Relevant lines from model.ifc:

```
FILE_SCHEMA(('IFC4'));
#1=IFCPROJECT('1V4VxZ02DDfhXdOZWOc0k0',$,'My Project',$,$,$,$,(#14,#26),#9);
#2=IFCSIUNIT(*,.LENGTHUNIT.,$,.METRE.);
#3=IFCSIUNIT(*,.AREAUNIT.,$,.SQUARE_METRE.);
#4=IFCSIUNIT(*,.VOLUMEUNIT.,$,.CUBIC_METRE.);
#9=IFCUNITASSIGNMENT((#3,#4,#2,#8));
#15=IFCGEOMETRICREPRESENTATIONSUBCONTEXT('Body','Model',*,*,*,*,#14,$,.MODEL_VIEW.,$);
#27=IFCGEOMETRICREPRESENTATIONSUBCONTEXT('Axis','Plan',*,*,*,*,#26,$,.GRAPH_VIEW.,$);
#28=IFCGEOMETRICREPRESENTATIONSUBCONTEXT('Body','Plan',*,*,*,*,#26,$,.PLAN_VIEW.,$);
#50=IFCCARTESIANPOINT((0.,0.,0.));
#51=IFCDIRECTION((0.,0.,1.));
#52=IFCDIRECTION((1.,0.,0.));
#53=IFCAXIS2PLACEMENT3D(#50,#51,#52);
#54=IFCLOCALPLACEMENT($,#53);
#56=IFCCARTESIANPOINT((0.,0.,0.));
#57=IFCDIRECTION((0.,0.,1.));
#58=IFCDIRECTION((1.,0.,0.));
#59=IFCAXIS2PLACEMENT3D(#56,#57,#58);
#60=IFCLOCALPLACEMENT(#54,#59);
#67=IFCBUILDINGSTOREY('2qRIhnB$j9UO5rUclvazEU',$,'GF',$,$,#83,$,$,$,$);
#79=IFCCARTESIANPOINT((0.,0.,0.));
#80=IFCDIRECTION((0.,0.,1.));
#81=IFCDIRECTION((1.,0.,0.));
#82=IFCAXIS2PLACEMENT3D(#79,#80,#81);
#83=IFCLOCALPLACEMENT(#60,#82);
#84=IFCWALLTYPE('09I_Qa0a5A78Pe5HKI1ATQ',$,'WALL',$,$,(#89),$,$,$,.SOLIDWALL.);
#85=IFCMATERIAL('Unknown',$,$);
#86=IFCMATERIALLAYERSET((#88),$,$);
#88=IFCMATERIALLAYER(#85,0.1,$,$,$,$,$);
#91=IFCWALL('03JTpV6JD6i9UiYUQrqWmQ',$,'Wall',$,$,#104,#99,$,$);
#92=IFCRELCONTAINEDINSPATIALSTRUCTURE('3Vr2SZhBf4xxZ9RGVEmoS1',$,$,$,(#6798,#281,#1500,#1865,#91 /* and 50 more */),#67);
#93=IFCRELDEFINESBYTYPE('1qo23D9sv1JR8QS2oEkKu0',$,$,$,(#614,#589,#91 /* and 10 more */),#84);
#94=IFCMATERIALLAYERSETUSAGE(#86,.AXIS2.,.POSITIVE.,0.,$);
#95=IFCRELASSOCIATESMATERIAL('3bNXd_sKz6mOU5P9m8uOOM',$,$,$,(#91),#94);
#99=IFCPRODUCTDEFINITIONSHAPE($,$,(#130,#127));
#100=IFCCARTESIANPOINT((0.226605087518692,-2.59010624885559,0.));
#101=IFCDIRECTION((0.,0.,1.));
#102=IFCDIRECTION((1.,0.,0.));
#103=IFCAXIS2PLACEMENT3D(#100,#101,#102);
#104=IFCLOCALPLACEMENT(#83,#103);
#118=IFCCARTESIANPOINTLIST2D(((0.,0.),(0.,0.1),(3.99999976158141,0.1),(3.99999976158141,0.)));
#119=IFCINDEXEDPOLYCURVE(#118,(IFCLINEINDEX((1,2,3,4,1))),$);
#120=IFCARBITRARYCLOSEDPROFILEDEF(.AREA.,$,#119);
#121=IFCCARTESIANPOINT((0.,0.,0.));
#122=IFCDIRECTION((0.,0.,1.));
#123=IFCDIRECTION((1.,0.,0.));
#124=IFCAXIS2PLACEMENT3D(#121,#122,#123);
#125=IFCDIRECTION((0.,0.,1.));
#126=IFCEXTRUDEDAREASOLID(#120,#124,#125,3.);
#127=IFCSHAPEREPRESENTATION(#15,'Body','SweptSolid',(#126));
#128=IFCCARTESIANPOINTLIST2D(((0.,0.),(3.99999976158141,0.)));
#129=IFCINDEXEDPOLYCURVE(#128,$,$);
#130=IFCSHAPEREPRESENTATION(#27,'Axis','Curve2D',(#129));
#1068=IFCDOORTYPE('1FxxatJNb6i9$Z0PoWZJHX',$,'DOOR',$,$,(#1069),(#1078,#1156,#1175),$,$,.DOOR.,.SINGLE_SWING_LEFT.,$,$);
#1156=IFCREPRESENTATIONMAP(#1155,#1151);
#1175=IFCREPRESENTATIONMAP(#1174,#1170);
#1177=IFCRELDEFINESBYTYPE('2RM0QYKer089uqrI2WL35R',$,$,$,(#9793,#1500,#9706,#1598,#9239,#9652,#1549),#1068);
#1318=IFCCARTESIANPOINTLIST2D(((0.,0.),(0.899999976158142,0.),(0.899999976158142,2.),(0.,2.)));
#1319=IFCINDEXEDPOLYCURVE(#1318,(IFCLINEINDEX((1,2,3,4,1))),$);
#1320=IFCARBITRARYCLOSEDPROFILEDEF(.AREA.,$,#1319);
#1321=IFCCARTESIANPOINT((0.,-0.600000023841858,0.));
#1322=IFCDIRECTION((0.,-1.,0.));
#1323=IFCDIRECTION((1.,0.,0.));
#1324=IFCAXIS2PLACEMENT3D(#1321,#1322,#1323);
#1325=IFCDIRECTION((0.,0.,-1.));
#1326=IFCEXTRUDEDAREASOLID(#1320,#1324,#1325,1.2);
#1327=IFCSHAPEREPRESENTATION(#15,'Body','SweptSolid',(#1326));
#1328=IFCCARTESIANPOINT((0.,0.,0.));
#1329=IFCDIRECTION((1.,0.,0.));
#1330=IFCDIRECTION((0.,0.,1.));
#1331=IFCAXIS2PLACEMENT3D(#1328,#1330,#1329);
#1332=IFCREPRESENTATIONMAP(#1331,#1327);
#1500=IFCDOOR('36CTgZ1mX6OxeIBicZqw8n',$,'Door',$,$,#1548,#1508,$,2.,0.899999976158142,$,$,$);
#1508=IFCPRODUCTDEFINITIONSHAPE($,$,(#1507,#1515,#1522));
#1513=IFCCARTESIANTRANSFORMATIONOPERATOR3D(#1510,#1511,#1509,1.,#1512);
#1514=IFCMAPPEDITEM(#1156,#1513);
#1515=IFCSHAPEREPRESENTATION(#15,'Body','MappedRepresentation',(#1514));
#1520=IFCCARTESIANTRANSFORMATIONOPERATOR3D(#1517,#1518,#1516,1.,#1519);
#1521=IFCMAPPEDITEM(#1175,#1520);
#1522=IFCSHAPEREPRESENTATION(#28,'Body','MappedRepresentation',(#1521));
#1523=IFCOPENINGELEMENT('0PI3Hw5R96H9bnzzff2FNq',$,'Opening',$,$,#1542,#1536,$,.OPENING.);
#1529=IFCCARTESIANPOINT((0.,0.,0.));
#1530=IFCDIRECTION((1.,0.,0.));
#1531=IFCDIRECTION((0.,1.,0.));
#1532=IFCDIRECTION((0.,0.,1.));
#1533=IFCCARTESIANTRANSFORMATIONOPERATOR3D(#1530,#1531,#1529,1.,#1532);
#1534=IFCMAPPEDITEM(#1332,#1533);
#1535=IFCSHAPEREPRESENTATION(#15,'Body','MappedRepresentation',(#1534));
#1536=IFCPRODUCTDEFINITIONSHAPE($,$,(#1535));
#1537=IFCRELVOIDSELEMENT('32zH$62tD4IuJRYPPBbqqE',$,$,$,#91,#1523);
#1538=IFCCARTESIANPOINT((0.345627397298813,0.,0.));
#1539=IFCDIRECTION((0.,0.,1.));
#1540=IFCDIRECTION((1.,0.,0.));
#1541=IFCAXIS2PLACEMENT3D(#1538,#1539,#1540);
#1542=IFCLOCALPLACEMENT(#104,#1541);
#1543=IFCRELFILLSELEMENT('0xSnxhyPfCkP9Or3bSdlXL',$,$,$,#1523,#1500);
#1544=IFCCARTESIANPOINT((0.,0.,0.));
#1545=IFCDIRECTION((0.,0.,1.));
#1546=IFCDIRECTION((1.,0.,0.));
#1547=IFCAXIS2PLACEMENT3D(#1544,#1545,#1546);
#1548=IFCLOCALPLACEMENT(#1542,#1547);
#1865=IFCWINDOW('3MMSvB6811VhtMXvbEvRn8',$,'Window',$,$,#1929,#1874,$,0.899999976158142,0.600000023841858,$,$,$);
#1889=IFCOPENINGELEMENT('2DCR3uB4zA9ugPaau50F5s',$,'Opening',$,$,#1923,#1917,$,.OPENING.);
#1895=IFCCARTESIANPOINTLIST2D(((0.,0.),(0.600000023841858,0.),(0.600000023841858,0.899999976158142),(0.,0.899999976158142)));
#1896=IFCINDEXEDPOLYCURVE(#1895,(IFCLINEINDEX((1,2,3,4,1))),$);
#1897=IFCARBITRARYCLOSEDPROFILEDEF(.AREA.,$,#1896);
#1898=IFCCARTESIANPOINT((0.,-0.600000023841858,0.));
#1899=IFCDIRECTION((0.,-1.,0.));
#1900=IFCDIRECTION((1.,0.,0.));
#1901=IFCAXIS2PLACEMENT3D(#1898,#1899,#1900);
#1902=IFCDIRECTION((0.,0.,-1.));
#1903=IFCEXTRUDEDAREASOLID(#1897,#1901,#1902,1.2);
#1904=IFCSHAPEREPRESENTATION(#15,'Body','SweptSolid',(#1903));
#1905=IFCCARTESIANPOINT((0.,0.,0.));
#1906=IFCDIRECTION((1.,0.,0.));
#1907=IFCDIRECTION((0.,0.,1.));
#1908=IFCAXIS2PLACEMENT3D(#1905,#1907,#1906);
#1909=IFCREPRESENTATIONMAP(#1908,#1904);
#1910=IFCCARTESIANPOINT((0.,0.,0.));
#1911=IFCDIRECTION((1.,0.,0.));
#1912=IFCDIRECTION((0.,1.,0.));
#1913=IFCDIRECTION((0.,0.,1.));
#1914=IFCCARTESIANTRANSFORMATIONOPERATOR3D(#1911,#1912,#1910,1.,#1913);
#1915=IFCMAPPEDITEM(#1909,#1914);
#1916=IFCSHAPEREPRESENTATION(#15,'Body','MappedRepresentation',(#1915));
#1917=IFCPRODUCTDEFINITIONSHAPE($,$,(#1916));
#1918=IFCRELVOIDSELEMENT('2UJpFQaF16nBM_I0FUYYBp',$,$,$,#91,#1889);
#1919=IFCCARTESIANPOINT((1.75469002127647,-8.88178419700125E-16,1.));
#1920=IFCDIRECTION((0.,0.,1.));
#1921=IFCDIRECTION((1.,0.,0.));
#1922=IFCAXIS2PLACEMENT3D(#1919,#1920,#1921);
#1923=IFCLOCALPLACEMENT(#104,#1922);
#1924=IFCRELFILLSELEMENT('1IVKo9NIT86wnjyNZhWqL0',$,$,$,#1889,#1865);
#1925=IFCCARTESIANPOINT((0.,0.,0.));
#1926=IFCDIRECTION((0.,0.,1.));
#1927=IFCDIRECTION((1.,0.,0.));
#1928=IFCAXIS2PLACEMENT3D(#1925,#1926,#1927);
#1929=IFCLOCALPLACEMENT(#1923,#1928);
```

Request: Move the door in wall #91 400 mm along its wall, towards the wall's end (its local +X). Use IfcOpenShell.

```python
import ifcopenshell
import ifcopenshell.api.geometry
import ifcopenshell.util.placement
import ifcopenshell.util.unit

model = ifcopenshell.open("model.ifc")
unit_scale = ifcopenshell.util.unit.calculate_unit_scale(model)

door = model.by_id(1500)
opening = door.FillsVoids[0].RelatingOpeningElement
wall = opening.VoidsElements[0].RelatingBuildingElement

wall_matrix = ifcopenshell.util.placement.get_local_placement(wall.ObjectPlacement)
shift = wall_matrix[:3, 0] * 0.4 / unit_scale
before = ifcopenshell.util.placement.get_local_placement(door.ObjectPlacement)[:3, 3].copy()

# The door is placed relative to its opening, so it follows when the opening moves.
matrix = ifcopenshell.util.placement.get_local_placement(opening.ObjectPlacement)
matrix[:3, 3] += shift
ifcopenshell.api.geometry.edit_object_placement(
    model, product=opening, matrix=matrix, is_si=False, should_transform_children=True
)

after = ifcopenshell.util.placement.get_local_placement(door.ObjectPlacement)[:3, 3]
print("door moved by", (after - before).round(3) + 0.0)

model.write("model_edited.ifc")
```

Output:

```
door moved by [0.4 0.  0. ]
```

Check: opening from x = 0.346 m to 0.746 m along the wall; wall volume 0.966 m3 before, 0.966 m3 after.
